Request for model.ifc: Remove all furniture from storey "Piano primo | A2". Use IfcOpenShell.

First a look at what the model holds.

```python
import ifcopenshell
import ifcopenshell.util.element

model = ifcopenshell.open("model.ifc")
print(model.schema)
storey = next(s for s in model.by_type("IfcBuildingStorey") if s.Name == "Piano primo | A2")
furniture = [e for e in ifcopenshell.util.element.get_decomposition(storey) if e.is_a("IfcFurnishingElement")]
seen = {}
for e in furniture:
    element_type = ifcopenshell.util.element.get_type(e)
    name = element_type.Name if element_type not in (None, e) else None
    seen[name] = seen.get(name, 0) + 1
for name, count in sorted(seen.items(), key=str):
    print(count, "x", name)
```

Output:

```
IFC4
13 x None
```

```python
import ifcopenshell
import ifcopenshell.api.root
import ifcopenshell.util.element

model = ifcopenshell.open("model.ifc")

storey = next(s for s in model.by_type("IfcBuildingStorey") if s.Name == "Piano primo | A2")
furniture = [e for e in ifcopenshell.util.element.get_decomposition(storey) if e.is_a("IfcFurnishingElement")]

for e in furniture:
    ifcopenshell.api.root.remove_product(model, product=e)
print(len(furniture), "removed")

model.write("model_v2.ifc")
```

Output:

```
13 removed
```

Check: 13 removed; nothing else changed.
